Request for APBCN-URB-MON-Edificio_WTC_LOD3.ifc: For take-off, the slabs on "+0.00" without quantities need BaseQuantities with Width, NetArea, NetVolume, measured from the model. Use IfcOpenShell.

First a look at what the model holds.

```python
import ifcopenshell
import ifcopenshell.util.element
import ifcopenshell.util.unit

model = ifcopenshell.open("APBCN-URB-MON-Edificio_WTC_LOD3.ifc")
print(model.schema)
for unit_type in ("LENGTHUNIT", "AREAUNIT", "VOLUMEUNIT"):
    print(unit_type, ifcopenshell.util.unit.calculate_unit_scale(model, unit_type))
storey = next(s for s in model.by_type("IfcBuildingStorey") if s.Name == "+0.00")
slabs = [e for e in ifcopenshell.util.element.get_decomposition(storey) if e.is_a("IfcSlab")]
for e in sorted(slabs, key=lambda e: e.id()):
    print(e.id(), e.is_a(), e.Name, list(ifcopenshell.util.element.get_psets(e, qtos_only=True)), sep=" | ")
```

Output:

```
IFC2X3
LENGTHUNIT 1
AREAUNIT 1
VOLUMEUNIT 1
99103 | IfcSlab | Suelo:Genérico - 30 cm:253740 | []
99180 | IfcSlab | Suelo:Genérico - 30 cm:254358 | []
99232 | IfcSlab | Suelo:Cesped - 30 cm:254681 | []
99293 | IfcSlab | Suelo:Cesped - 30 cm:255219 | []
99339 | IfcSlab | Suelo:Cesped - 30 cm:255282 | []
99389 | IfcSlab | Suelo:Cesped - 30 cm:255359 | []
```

```python
import ifcopenshell
import ifcopenshell.api.pset
import ifcopenshell.geom
import ifcopenshell.util.element
import ifcopenshell.util.shape
import ifcopenshell.util.unit

model = ifcopenshell.open("APBCN-URB-MON-Edificio_WTC_LOD3.ifc")
unit_scale = ifcopenshell.util.unit.calculate_unit_scale(model)
area_scale = ifcopenshell.util.unit.calculate_unit_scale(model, "AREAUNIT")
volume_scale = ifcopenshell.util.unit.calculate_unit_scale(model, "VOLUMEUNIT")
settings = ifcopenshell.geom.settings()

storey = next(s for s in model.by_type("IfcBuildingStorey") if s.Name == "+0.00")
slabs = [e for e in ifcopenshell.util.element.get_decomposition(storey) if e.is_a("IfcSlab")]

for e in sorted(slabs, key=lambda e: e.id()):
    if ifcopenshell.util.element.get_psets(e, qtos_only=True, should_inherit=False):
        continue
    # Geometry comes back in metres, in the element's own axes.
    shape = ifcopenshell.geom.create_shape(settings, e)
    values = {
        "Width": ifcopenshell.util.shape.get_z(shape.geometry) / unit_scale,
        "NetArea": ifcopenshell.util.shape.get_footprint_area(shape.geometry) / area_scale,
        "NetVolume": ifcopenshell.util.shape.get_volume(shape.geometry) / volume_scale,
    }
    qto = ifcopenshell.api.pset.add_qto(model, product=e, name="BaseQuantities")
    ifcopenshell.api.pset.edit_qto(model, qto=qto, properties=values)
    print(e.id(), {k: round(v, 3) for k, v in values.items()})

model.write("APBCN-URB-MON-Edificio_WTC_LOD3_rev.ifc")
```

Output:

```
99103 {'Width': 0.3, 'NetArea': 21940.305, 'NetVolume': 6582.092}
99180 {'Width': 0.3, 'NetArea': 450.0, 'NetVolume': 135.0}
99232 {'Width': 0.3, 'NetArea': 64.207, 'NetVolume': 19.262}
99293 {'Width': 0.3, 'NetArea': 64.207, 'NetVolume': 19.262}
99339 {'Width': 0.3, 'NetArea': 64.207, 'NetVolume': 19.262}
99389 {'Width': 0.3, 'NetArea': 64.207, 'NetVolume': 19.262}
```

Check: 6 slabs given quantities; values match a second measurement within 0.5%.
